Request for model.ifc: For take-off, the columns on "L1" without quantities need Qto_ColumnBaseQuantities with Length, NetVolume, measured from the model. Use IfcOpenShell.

First a look at what the model holds.

```python
import ifcopenshell
import ifcopenshell.util.element
import ifcopenshell.util.unit

model = ifcopenshell.open("model.ifc")
print(model.schema)
for unit_type in ("LENGTHUNIT", "AREAUNIT", "VOLUMEUNIT"):
    print(unit_type, ifcopenshell.util.unit.calculate_unit_scale(model, unit_type))
storey = next(s for s in model.by_type("IfcBuildingStorey") if s.Name == "L1")
columns = [e for e in ifcopenshell.util.element.get_decomposition(storey) if e.is_a("IfcColumn")]
for e in sorted(columns, key=lambda e: e.id()):
    print(e.id(), e.is_a(), e.Name, list(ifcopenshell.util.element.get_psets(e, qtos_only=True)), sep=" | ")
```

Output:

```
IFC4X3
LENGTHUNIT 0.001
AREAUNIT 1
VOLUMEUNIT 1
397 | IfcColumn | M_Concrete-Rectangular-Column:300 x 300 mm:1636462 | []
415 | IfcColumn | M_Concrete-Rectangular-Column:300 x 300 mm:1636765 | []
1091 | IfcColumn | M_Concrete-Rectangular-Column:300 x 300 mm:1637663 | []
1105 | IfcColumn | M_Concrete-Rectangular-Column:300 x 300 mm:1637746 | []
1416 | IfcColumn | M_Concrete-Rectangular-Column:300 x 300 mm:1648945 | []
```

```python
import ifcopenshell
import ifcopenshell.api.pset
import ifcopenshell.geom
import ifcopenshell.util.element
import ifcopenshell.util.shape
import ifcopenshell.util.unit

model = ifcopenshell.open("model.ifc")
unit_scale = ifcopenshell.util.unit.calculate_unit_scale(model)
volume_scale = ifcopenshell.util.unit.calculate_unit_scale(model, "VOLUMEUNIT")
settings = ifcopenshell.geom.settings()

storey = next(s for s in model.by_type("IfcBuildingStorey") if s.Name == "L1")
columns = [e for e in ifcopenshell.util.element.get_decomposition(storey) if e.is_a("IfcColumn")]

for e in sorted(columns, key=lambda e: e.id()):
    if ifcopenshell.util.element.get_psets(e, qtos_only=True, should_inherit=False):
        continue
    # Geometry comes back in metres, in the element's own axes.
    shape = ifcopenshell.geom.create_shape(settings, e)
    values = {
        "Length": ifcopenshell.util.shape.get_z(shape.geometry) / unit_scale,
        "NetVolume": ifcopenshell.util.shape.get_volume(shape.geometry) / volume_scale,
    }
    qto = ifcopenshell.api.pset.add_qto(model, product=e, name="Qto_ColumnBaseQuantities")
    ifcopenshell.api.pset.edit_qto(model, qto=qto, properties=values)
    print(e.id(), {k: round(v, 3) for k, v in values.items()})

model.write("model-out.ifc")
```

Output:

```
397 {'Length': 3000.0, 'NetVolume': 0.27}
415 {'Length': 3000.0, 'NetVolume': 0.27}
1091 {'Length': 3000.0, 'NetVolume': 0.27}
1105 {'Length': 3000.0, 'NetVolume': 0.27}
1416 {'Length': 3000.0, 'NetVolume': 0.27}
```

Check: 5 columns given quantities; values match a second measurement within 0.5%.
